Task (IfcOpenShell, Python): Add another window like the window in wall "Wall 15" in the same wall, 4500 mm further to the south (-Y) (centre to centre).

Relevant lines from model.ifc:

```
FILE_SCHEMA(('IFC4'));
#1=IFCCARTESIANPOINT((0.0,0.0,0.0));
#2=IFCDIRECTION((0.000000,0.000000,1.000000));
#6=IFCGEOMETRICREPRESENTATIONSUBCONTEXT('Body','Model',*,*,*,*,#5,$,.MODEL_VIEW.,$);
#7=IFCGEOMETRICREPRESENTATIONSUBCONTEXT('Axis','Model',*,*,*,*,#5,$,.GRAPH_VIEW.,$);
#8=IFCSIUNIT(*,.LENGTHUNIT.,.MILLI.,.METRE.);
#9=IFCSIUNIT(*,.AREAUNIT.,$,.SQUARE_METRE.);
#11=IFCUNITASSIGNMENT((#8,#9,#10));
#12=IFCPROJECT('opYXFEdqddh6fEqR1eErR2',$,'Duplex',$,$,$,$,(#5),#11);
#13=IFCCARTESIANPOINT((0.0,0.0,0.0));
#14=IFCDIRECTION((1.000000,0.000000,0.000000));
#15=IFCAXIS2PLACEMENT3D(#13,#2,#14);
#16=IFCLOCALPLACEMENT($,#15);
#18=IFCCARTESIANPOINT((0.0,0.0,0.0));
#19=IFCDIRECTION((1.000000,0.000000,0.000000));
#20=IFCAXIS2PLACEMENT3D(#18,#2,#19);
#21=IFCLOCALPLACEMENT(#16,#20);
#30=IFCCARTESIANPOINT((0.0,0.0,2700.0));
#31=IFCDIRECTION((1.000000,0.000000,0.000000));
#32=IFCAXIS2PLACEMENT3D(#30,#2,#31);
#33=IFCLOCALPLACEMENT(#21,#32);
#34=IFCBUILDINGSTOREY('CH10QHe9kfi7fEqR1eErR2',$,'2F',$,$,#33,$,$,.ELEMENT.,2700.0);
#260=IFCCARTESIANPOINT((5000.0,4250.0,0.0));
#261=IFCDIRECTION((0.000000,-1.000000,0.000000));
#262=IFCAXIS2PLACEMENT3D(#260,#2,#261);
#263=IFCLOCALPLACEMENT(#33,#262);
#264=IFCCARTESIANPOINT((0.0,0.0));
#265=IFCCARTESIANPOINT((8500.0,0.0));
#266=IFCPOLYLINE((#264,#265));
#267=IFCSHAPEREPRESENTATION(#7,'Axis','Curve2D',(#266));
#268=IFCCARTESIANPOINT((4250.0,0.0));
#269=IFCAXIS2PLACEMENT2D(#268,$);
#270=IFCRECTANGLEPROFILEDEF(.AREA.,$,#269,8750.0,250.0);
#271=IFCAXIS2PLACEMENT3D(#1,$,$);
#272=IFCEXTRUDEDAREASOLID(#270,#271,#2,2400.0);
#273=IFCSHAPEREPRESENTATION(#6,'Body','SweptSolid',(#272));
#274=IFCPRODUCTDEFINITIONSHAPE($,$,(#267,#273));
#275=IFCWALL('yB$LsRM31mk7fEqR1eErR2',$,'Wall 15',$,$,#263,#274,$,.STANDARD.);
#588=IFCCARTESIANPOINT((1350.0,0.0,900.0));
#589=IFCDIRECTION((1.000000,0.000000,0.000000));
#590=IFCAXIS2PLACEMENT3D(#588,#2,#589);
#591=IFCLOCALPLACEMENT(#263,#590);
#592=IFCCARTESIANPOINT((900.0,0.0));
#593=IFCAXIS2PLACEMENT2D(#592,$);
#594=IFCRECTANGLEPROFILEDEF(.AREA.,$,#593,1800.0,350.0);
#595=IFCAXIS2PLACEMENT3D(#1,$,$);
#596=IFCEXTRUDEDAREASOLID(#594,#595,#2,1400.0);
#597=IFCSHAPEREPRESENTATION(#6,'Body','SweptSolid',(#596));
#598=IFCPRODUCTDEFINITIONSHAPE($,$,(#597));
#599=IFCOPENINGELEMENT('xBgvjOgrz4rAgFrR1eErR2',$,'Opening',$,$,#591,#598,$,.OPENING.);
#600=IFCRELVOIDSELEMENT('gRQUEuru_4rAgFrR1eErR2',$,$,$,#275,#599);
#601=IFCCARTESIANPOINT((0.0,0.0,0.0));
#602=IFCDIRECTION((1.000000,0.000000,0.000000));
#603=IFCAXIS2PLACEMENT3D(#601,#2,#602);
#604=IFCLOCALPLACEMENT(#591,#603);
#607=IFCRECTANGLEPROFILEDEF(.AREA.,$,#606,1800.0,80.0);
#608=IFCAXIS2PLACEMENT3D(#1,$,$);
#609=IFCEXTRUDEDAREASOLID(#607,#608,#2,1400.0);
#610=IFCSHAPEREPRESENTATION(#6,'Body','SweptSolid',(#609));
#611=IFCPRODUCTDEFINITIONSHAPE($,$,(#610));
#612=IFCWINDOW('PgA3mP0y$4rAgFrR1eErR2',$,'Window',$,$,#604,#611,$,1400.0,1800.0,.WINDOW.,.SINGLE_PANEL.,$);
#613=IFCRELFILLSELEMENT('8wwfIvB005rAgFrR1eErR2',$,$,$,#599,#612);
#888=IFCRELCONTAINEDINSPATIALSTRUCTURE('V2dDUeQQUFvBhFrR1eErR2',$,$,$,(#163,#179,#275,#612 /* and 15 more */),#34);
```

```python
import ifcopenshell
import ifcopenshell.api.feature
import ifcopenshell.api.geometry
import ifcopenshell.api.root
import ifcopenshell.geom
import ifcopenshell.util.element
import ifcopenshell.util.placement
import ifcopenshell.util.shape
import ifcopenshell.util.unit

model = ifcopenshell.open("model.ifc")
unit_scale = ifcopenshell.util.unit.calculate_unit_scale(model)
settings = ifcopenshell.geom.settings()


def volume(element):
    """Net volume in cubic metres, openings subtracted."""
    shape = ifcopenshell.geom.create_shape(settings, element)
    return ifcopenshell.util.shape.get_volume(shape.geometry)


window = model.by_guid("PgA3mP0y$4rAgFrR1eErR2")
opening = window.FillsVoids[0].RelatingOpeningElement
wall = opening.VoidsElements[0].RelatingBuildingElement
before = volume(wall)
shift = ifcopenshell.util.placement.get_local_placement(wall.ObjectPlacement)[:3, 0] * 4.5 / unit_scale

# copy_class copies the void relationship, type, container and properties, but no geometry.
new_opening = ifcopenshell.api.root.copy_class(model, product=opening)
new_opening.Representation = ifcopenshell.util.element.copy_deep(
    model, opening.Representation, exclude=["IfcGeometricRepresentationContext", "IfcRepresentationMap"]
)
new_window = ifcopenshell.api.root.copy_class(model, product=window)
new_window.Representation = ifcopenshell.util.element.copy_deep(
    model, window.Representation, exclude=["IfcGeometricRepresentationContext", "IfcRepresentationMap"]
)
ifcopenshell.api.feature.add_filling(model, opening=new_opening, element=new_window)

for old, new in ((opening, new_opening), (window, new_window)):
    matrix = ifcopenshell.util.placement.get_local_placement(old.ObjectPlacement)
    matrix[:3, 3] += shift
    ifcopenshell.api.geometry.edit_object_placement(model, product=new, matrix=matrix, is_si=False)

after = volume(wall)

print(f"wall volume {before:.3f} -> {after:.3f} m3")

model.write("model_edited.ifc")
```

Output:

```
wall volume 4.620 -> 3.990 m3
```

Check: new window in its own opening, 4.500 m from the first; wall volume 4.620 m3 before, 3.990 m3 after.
